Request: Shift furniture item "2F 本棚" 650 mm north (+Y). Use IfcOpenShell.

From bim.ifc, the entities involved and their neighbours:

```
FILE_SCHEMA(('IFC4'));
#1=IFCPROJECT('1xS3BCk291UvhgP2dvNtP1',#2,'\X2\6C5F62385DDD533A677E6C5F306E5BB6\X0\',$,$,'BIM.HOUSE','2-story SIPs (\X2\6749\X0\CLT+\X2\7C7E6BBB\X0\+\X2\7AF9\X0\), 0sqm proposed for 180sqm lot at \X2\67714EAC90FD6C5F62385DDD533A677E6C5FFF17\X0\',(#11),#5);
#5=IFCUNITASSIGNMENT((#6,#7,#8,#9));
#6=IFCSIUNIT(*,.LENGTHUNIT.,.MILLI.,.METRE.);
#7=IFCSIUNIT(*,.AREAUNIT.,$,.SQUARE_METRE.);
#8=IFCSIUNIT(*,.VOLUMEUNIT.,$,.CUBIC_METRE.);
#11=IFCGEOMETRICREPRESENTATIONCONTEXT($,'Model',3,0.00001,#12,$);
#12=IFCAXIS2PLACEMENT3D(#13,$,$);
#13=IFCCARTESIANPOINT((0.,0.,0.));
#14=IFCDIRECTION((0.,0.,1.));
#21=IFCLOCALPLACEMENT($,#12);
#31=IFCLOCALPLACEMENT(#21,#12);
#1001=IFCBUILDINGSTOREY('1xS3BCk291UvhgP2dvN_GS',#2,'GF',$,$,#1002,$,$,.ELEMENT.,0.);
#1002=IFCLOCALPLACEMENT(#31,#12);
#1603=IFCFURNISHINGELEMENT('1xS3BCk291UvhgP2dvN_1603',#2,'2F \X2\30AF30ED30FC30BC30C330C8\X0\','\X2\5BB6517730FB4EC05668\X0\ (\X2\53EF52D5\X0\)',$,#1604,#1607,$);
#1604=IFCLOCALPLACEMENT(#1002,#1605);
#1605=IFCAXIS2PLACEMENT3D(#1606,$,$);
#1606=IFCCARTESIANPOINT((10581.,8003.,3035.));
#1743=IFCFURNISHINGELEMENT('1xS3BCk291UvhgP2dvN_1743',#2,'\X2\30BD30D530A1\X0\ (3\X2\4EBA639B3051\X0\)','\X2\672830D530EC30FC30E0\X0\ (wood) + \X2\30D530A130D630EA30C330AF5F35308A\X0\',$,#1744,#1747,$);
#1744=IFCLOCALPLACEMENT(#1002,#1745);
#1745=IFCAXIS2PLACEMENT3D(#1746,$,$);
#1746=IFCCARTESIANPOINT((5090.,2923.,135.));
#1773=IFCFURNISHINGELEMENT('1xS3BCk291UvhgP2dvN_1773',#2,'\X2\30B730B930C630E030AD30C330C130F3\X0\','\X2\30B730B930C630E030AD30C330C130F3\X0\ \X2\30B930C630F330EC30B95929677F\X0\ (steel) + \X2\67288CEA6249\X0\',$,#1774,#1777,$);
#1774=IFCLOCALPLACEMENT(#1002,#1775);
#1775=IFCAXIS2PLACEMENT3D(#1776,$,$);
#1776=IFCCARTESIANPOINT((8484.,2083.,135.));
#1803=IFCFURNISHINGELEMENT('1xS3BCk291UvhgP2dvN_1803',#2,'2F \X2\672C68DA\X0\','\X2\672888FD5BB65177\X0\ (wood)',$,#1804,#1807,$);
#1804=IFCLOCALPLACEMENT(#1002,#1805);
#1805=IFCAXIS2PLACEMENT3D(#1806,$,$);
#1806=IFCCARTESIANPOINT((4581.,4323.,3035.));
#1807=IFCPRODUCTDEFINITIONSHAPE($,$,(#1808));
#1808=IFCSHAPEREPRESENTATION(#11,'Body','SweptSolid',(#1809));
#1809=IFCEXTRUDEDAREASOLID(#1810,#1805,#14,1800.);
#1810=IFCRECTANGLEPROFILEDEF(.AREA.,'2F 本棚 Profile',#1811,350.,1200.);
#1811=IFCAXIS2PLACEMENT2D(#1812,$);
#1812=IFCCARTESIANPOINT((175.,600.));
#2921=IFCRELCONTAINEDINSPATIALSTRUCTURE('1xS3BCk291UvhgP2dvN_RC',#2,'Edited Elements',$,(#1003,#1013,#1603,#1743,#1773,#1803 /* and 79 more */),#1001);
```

```python
import ifcopenshell
import ifcopenshell.api.geometry
import ifcopenshell.util.placement

model = ifcopenshell.open("bim.ifc")

item = model.by_guid("1xS3BCk291UvhgP2dvN_1803")
matrix = ifcopenshell.util.placement.get_local_placement(item.ObjectPlacement)
matrix[1, 3] += 650.0
ifcopenshell.api.geometry.edit_object_placement(model, product=item, matrix=matrix, is_si=False)

print(ifcopenshell.util.placement.get_local_placement(item.ObjectPlacement).round(3) + 0.0)

model.write("bim_v2.ifc")
```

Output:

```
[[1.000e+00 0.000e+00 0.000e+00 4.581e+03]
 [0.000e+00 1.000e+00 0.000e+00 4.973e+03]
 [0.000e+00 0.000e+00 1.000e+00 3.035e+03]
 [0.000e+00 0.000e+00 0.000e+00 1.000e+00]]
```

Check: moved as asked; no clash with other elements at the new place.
